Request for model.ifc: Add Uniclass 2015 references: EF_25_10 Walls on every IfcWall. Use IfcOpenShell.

First a look at what the model holds.

```python
import ifcopenshell

model = ifcopenshell.open("model.ifc")
print(model.schema)
print("classifications:", [c.Name for c in model.by_type("IfcClassification")])
for ifc_class in ("IfcDoor", "IfcRoof", "IfcStair", "IfcWall", "IfcWindow"):
    print(ifc_class, len(model.by_type(ifc_class)))
```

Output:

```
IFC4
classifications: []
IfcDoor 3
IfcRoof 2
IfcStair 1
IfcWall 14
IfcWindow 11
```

```python
import ifcopenshell
import ifcopenshell.api.classification

model = ifcopenshell.open("model.ifc")

system = ifcopenshell.api.classification.add_classification(model, classification="Uniclass 2015")

codes = {
    "IfcWall": ("EF_25_10", "Walls"),
}
for ifc_class, (code, name) in codes.items():
    products = model.by_type(ifc_class)
    ifcopenshell.api.classification.add_reference(
        model, products=products, classification=system, identification=code, name=name
    )
    print(code, len(products))

model.write("model-out.ifc")
```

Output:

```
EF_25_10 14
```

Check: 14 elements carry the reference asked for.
